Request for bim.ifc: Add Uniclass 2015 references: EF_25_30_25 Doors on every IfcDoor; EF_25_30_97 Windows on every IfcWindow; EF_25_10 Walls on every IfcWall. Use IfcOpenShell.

First a look at what the model holds.

```python
import ifcopenshell

model = ifcopenshell.open("bim.ifc")
print(model.schema)
print("classifications:", [c.Name for c in model.by_type("IfcClassification")])
for ifc_class in ("IfcDoor", "IfcRoof", "IfcStair", "IfcWall", "IfcWindow"):
    print(ifc_class, len(model.by_type(ifc_class)))
```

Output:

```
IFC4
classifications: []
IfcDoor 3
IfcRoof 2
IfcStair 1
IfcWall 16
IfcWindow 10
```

```python
import ifcopenshell
import ifcopenshell.api.classification

model = ifcopenshell.open("bim.ifc")

system = ifcopenshell.api.classification.add_classification(model, classification="Uniclass 2015")

codes = {
    "IfcDoor": ("EF_25_30_25", "Doors"),
    "IfcWindow": ("EF_25_30_97", "Windows"),
    "IfcWall": ("EF_25_10", "Walls"),
}
for ifc_class, (code, name) in codes.items():
    products = model.by_type(ifc_class)
    ifcopenshell.api.classification.add_reference(
        model, products=products, classification=system, identification=code, name=name
    )
    print(code, len(products))

model.write("bim-out.ifc")
```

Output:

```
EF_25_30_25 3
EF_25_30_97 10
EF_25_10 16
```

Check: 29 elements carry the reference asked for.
